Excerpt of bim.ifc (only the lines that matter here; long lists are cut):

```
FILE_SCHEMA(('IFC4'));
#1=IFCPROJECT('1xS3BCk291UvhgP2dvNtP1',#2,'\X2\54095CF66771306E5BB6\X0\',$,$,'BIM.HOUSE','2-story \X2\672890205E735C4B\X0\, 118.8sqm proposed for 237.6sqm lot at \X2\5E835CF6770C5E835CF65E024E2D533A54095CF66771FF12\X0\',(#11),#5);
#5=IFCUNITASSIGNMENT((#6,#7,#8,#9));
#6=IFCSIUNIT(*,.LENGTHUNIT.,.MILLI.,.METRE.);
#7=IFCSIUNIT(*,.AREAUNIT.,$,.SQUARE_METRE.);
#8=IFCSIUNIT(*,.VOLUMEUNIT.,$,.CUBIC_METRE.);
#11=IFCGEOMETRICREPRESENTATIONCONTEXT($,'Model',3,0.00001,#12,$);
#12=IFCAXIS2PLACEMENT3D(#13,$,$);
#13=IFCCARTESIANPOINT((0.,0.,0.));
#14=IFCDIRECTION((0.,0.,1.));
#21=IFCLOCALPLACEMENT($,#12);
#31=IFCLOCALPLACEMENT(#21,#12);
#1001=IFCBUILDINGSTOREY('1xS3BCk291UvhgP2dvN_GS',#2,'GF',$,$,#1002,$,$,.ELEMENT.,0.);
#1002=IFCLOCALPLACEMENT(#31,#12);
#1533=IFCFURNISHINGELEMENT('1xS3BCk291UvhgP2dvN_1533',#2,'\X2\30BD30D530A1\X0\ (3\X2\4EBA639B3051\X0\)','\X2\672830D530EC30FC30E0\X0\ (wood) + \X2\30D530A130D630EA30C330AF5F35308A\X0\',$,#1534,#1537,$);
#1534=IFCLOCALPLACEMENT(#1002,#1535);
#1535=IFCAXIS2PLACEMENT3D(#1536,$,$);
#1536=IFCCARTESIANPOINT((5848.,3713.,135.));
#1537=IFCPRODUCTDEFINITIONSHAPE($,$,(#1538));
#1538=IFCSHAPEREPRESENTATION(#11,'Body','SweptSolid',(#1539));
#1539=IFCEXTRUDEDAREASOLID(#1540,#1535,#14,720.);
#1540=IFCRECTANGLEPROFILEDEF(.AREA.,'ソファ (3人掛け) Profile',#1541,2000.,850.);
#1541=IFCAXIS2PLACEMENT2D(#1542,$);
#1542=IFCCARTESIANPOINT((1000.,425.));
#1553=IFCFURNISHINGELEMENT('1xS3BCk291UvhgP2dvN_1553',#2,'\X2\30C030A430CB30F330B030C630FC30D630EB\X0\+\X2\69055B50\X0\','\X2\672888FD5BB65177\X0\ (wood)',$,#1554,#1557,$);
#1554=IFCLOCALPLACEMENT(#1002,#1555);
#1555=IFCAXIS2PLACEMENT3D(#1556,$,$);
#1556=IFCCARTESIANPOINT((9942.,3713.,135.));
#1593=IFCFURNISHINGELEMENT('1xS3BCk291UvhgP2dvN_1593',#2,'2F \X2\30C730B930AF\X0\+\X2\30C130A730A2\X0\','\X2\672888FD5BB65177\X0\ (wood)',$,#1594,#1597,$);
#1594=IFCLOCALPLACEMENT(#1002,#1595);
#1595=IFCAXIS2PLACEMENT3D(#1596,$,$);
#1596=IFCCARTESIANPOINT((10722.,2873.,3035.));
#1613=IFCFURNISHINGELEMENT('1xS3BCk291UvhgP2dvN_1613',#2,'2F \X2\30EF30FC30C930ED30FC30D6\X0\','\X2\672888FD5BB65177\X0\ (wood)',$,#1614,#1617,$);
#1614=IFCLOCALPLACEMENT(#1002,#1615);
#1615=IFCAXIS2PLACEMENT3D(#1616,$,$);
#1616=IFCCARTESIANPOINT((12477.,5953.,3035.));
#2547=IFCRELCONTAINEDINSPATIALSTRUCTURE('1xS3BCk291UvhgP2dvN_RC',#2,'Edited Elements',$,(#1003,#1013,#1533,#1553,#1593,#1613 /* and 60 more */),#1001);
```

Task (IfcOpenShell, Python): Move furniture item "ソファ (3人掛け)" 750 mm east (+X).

```python
import ifcopenshell
import ifcopenshell.api.geometry
import ifcopenshell.util.placement
import ifcopenshell.util.unit

model = ifcopenshell.open("bim.ifc")
unit_scale = ifcopenshell.util.unit.calculate_unit_scale(model)

item = model.by_guid("1xS3BCk291UvhgP2dvN_1533")
matrix = ifcopenshell.util.placement.get_local_placement(item.ObjectPlacement)
matrix[0, 3] += 0.75 / unit_scale
ifcopenshell.api.geometry.edit_object_placement(model, product=item, matrix=matrix, is_si=False)

print(ifcopenshell.util.placement.get_local_placement(item.ObjectPlacement).round(3) + 0.0)

model.write("bim_updated.ifc")
```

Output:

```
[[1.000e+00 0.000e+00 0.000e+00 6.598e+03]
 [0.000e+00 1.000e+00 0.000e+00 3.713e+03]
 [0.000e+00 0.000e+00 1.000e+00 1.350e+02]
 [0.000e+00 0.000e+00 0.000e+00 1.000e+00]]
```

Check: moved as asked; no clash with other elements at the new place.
